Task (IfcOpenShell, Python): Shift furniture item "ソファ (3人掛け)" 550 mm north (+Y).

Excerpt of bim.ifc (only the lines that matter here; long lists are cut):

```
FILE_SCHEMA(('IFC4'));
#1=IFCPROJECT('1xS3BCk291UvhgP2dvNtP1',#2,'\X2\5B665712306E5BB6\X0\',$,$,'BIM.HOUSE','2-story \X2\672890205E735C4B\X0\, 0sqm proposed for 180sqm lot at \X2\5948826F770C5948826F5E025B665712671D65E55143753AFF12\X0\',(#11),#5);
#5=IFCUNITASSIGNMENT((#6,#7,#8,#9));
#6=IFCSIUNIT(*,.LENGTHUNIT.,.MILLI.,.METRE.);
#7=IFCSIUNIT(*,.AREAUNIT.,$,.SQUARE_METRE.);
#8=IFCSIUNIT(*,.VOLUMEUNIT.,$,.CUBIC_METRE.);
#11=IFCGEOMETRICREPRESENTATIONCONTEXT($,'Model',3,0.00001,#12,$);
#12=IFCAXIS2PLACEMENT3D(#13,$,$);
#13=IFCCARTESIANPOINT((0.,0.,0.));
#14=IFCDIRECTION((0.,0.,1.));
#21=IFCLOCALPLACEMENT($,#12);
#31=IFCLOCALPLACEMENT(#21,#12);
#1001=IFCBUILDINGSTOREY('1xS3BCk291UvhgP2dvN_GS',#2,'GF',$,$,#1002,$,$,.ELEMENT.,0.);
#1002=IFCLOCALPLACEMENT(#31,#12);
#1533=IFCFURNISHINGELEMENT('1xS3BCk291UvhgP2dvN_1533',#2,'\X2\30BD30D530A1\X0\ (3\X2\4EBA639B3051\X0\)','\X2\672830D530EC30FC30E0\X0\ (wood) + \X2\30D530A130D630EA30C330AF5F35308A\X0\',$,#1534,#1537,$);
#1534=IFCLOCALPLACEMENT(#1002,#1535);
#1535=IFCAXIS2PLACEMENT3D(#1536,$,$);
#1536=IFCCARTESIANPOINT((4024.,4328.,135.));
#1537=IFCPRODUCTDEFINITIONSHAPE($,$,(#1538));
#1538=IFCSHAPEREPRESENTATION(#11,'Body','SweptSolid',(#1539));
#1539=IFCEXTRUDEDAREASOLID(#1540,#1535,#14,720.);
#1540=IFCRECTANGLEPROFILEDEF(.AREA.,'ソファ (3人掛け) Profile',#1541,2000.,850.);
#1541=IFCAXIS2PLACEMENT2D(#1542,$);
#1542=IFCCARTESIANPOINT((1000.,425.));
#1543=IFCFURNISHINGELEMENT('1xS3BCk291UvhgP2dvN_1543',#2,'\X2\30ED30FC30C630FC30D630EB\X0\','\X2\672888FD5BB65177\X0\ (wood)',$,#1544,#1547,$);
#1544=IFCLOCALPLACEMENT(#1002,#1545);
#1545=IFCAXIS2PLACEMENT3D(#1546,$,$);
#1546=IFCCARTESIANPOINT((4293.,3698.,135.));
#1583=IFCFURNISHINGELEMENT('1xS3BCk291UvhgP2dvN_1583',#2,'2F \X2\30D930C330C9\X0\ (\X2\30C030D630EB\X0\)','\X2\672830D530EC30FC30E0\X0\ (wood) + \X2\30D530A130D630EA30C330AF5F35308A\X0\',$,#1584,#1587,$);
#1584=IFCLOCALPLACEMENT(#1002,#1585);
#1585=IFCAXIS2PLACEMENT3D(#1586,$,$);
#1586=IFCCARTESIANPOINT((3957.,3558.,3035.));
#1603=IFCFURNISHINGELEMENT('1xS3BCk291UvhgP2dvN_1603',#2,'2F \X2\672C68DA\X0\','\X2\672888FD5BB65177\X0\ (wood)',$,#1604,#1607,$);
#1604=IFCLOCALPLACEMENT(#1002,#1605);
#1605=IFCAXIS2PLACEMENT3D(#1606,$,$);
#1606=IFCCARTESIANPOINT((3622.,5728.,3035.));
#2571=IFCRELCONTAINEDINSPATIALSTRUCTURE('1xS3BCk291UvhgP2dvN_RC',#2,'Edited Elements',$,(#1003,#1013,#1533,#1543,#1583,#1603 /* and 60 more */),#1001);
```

```python
import ifcopenshell
import ifcopenshell.api.geometry
import ifcopenshell.util.placement

model = ifcopenshell.open("bim.ifc")

item = model.by_guid("1xS3BCk291UvhgP2dvN_1533")
matrix = ifcopenshell.util.placement.get_local_placement(item.ObjectPlacement)
matrix[1, 3] += 550.0
ifcopenshell.api.geometry.edit_object_placement(model, product=item, matrix=matrix, is_si=False)

print(ifcopenshell.util.placement.get_local_placement(item.ObjectPlacement).round(3) + 0.0)

model.write("bim-out.ifc")
```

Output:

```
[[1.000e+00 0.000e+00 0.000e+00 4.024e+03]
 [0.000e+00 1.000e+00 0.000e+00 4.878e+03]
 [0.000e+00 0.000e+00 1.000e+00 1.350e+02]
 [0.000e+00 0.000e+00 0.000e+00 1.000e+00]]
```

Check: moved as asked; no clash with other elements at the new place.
